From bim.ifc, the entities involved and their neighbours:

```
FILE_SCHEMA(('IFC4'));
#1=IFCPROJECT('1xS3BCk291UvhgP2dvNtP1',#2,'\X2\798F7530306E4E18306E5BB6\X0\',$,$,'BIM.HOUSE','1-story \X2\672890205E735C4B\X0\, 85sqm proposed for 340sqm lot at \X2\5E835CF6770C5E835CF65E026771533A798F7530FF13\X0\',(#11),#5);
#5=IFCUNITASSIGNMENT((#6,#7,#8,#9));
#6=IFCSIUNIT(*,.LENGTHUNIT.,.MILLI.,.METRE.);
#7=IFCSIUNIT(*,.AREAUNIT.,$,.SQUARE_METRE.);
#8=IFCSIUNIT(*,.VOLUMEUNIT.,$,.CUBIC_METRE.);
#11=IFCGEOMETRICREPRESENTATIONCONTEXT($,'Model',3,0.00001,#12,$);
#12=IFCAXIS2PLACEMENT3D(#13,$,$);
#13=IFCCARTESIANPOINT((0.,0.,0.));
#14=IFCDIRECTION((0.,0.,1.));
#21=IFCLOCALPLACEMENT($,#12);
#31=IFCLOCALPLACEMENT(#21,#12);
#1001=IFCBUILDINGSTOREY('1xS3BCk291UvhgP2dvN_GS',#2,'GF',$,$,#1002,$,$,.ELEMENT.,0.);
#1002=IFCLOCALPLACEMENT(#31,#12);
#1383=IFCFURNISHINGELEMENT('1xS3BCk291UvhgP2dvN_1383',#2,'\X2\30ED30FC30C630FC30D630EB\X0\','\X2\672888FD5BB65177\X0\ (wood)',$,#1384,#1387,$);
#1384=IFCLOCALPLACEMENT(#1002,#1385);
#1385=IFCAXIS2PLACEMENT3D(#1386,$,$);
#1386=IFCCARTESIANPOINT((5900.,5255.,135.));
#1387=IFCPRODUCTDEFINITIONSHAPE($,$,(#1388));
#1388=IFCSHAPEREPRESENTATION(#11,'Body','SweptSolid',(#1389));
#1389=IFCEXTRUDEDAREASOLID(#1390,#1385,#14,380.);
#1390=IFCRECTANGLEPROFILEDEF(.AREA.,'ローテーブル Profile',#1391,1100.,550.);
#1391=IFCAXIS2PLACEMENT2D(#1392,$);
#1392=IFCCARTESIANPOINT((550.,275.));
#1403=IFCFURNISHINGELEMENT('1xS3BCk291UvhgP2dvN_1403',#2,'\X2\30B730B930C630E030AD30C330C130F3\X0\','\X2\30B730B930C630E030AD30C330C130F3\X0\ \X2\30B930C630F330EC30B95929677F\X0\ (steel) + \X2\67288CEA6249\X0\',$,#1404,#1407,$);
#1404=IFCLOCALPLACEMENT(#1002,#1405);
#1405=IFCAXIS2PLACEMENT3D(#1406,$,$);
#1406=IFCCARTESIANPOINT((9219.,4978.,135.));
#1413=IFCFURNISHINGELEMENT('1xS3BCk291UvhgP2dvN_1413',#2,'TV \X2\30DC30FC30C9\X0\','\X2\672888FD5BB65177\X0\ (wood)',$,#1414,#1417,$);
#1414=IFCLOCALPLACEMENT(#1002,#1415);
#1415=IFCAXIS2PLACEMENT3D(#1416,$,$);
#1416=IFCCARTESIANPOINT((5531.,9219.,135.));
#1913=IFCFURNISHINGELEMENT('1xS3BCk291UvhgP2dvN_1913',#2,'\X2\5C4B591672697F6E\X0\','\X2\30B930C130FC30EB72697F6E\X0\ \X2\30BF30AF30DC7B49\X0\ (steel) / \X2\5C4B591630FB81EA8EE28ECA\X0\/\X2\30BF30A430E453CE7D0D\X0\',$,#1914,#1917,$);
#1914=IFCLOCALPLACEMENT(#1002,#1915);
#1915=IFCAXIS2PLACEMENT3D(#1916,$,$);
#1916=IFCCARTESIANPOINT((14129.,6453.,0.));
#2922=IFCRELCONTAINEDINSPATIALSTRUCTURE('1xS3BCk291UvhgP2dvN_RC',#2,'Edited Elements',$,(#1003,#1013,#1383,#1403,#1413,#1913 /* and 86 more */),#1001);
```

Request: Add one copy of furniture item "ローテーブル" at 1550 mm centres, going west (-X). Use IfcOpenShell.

```python
import numpy as np
import ifcopenshell
import ifcopenshell.api.geometry
import ifcopenshell.api.root
import ifcopenshell.util.element
import ifcopenshell.util.placement
import ifcopenshell.util.unit

model = ifcopenshell.open("bim.ifc")
unit_scale = ifcopenshell.util.unit.calculate_unit_scale(model)


def reuse_history(source, copy):
    """copy_class also copies each property set's owner history, people and application; keep the originals."""
    for rel in copy.IsDefinedBy:
        if rel.is_a("IfcRelDefinesByProperties") and (history := rel.RelatingPropertyDefinition.OwnerHistory):
            rel.RelatingPropertyDefinition.OwnerHistory = source.OwnerHistory
            ifcopenshell.util.element.remove_deep2(model, history)


source = model.by_guid("1xS3BCk291UvhgP2dvN_1383")
base = ifcopenshell.util.placement.get_local_placement(source.ObjectPlacement)
step = np.array([-1.0, 0.0, 0.0]) * 1.55 / unit_scale

for i in range(1, 2):
    copy = ifcopenshell.api.root.copy_class(model, product=source)
    copy.Representation = ifcopenshell.util.element.copy_deep(
        model, source.Representation, exclude=["IfcGeometricRepresentationContext", "IfcRepresentationMap"]
    )
    reuse_history(source, copy)
    matrix = base.copy()
    matrix[:3, 3] += i * step
    print("added at", matrix[:3, 3].round(3) + 0.0)
    ifcopenshell.api.geometry.edit_object_placement(model, product=copy, matrix=matrix, is_si=False)

model.write("bim_edited.ifc")
```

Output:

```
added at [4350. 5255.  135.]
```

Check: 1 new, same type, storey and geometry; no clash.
